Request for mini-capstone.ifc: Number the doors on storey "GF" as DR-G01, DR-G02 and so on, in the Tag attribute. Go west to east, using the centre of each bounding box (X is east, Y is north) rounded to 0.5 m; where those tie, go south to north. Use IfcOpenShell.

First a look at what the model holds.

```python
import ifcopenshell
import ifcopenshell.util.element
import ifcopenshell.util.placement

model = ifcopenshell.open("mini-capstone.ifc")
print(model.schema)
storey = next(s for s in model.by_type("IfcBuildingStorey") if s.Name == "GF")
doors = [e for e in ifcopenshell.util.element.get_decomposition(storey) if e.is_a("IfcDoor")]
for e in sorted(doors, key=lambda e: e.id()):
    origin = ifcopenshell.util.placement.get_local_placement(e.ObjectPlacement)[:3, 3]
    print(e.id(), e.Tag, e.Name, origin.round(2) + 0.0, sep=" | ")
```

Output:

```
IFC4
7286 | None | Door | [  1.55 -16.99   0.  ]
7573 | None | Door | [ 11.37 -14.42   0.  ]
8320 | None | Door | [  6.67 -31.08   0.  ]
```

```python
import ifcopenshell
import ifcopenshell.geom
import ifcopenshell.util.element
import ifcopenshell.util.shape

model = ifcopenshell.open("mini-capstone.ifc")
settings = ifcopenshell.geom.settings()
settings.set("use-world-coords", True)


def centre(element):
    shape = ifcopenshell.geom.create_shape(settings, element)
    return ifcopenshell.util.shape.get_bbox_centroid(shape.geometry)


storey = next(s for s in model.by_type("IfcBuildingStorey") if s.Name == "GF")
doors = [e for e in ifcopenshell.util.element.get_decomposition(storey) if e.is_a("IfcDoor")]

# Insertion points can sit at a corner or the storey origin, so sort by the geometry (in metres).
centres = {e: centre(e) for e in doors}
doors.sort(key=lambda e: (round(centres[e][0] / 0.5), centres[e][1]))

for i, e in enumerate(doors, start=1):
    number = f"DR-G{i:02d}"
    e.Tag = number
    print(e.id(), number)

model.write("mini-capstone_updated.ifc")
```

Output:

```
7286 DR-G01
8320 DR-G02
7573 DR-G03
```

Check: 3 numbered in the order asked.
